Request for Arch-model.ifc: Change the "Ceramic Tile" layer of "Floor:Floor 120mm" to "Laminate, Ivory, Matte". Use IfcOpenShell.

First a look at what the model holds.

```python
import ifcopenshell
import ifcopenshell.util.element

model = ifcopenshell.open("Arch-model.ifc")
print(model.schema)
for layer_set in model.by_type("IfcMaterialLayerSet"):
    if layer_set.LayerSetName == "Floor:Floor 120mm":
        for layer in layer_set.MaterialLayers:
            print(layer.id(), layer.Material and layer.Material.Name, layer.LayerThickness, sep=" | ")
        print(len(ifcopenshell.util.element.get_elements_by_material(model, layer_set)), "elements and types use it")
print(sorted(m.Name for m in model.by_type("IfcMaterial") if m.Name)[:60])
```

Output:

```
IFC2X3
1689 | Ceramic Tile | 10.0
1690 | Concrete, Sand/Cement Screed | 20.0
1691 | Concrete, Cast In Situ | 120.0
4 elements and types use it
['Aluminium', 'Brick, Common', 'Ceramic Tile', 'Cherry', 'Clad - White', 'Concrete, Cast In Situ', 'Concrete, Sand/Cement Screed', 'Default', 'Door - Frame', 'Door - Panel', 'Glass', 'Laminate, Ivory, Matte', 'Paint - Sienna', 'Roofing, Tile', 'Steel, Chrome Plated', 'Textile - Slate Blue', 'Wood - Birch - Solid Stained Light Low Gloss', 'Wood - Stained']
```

```python
import ifcopenshell
import ifcopenshell.api.material

model = ifcopenshell.open("Arch-model.ifc")

layer_set = next(s for s in model.by_type("IfcMaterialLayerSet") if s.LayerSetName == "Floor:Floor 120mm")
layer = next(l for l in layer_set.MaterialLayers if l.Material and l.Material.Name == "Ceramic Tile")
material = next(m for m in model.by_type("IfcMaterial") if m.Name == "Laminate, Ivory, Matte")

# Point this one layer at the other material; renaming the old one would change it everywhere.
ifcopenshell.api.material.edit_layer(model, layer=layer, attributes={}, material=material)

print([l.Material.Name if l.Material else None for l in layer_set.MaterialLayers])

model.write("Arch-model_v2.ifc")
```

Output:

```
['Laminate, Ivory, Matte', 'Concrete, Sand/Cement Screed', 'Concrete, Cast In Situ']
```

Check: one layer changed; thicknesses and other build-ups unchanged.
